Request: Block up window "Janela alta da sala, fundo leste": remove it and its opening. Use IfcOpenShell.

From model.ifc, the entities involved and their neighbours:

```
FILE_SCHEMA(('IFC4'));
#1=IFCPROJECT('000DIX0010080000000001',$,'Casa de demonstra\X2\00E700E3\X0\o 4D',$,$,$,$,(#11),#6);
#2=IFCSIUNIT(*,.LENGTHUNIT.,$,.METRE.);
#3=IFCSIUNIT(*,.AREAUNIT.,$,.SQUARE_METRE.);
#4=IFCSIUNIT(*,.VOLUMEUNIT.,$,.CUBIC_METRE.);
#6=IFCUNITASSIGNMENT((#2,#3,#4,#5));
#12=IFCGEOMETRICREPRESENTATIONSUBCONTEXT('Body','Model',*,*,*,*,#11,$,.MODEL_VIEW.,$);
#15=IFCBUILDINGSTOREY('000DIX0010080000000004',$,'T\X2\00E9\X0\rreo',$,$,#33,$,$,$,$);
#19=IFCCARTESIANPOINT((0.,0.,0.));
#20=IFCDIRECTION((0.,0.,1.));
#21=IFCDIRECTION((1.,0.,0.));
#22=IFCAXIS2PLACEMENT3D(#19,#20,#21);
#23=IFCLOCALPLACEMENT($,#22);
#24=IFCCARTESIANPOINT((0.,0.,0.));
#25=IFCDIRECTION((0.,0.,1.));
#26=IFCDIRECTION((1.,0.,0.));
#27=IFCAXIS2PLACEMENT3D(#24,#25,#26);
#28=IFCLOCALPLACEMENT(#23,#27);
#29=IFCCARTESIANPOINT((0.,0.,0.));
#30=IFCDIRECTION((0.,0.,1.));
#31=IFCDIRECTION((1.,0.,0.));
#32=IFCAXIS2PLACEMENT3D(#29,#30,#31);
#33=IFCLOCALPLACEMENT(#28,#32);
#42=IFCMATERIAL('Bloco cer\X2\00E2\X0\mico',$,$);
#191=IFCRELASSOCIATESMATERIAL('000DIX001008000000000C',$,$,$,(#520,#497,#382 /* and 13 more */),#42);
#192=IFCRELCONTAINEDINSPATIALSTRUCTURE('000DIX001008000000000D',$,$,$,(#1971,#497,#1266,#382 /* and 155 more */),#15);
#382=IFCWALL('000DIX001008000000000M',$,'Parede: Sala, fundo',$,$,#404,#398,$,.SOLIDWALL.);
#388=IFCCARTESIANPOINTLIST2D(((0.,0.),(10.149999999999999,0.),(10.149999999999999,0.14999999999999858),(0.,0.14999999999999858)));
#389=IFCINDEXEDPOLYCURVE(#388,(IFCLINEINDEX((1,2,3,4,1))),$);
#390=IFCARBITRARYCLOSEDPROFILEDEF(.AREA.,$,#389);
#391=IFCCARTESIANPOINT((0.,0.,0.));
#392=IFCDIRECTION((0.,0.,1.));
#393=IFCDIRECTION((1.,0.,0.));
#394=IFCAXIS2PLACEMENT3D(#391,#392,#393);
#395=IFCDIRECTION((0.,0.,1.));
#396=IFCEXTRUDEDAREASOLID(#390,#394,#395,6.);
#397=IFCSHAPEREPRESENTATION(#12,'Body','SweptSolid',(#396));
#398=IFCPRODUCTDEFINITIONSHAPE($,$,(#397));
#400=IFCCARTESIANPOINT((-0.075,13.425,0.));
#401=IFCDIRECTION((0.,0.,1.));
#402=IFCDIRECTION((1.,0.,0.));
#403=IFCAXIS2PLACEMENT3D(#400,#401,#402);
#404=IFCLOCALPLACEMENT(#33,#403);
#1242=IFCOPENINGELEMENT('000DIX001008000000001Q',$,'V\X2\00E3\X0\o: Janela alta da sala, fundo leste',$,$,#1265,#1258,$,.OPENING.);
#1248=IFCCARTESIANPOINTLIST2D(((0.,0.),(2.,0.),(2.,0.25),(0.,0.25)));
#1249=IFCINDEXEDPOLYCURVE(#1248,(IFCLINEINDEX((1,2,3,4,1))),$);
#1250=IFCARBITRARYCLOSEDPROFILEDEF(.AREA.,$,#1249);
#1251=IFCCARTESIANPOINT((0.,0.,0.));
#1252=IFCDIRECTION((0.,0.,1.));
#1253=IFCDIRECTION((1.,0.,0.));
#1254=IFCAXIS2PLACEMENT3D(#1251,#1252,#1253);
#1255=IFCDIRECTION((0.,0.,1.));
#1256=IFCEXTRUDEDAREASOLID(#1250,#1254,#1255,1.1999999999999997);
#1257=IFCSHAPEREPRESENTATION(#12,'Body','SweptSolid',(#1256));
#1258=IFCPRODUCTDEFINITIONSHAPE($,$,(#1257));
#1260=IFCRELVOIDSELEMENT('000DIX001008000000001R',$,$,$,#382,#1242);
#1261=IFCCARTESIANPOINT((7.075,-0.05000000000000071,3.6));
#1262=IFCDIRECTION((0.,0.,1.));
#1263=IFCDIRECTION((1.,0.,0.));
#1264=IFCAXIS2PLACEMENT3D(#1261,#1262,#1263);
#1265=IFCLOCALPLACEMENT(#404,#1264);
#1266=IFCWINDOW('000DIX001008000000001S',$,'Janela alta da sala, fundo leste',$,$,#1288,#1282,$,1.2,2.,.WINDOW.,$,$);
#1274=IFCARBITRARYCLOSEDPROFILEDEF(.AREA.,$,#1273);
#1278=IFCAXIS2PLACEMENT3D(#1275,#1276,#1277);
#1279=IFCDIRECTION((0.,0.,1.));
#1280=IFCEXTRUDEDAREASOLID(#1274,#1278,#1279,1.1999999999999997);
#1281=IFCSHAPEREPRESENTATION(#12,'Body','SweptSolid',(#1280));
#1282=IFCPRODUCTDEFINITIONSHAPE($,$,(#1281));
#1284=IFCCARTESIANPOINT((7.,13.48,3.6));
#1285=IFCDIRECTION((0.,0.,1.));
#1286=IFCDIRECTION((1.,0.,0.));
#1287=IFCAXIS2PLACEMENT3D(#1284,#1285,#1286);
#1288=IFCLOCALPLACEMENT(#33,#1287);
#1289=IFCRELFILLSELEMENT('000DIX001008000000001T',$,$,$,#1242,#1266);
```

```python
import ifcopenshell
import ifcopenshell.api.feature
import ifcopenshell.api.root
import ifcopenshell.geom
import ifcopenshell.util.shape

model = ifcopenshell.open("model.ifc")
settings = ifcopenshell.geom.settings()


def volume(element):
    """Net volume in cubic metres, openings subtracted."""
    shape = ifcopenshell.geom.create_shape(settings, element)
    return ifcopenshell.util.shape.get_volume(shape.geometry)


window = model.by_guid("000DIX001008000000001S")
opening = window.FillsVoids[0].RelatingOpeningElement
wall = opening.VoidsElements[0].RelatingBuildingElement
before = volume(wall)

ifcopenshell.api.root.remove_product(model, product=window)
ifcopenshell.api.feature.remove_feature(model, feature=opening)

after = volume(wall)

print(f"wall volume {before:.3f} -> {after:.3f} m3")

model.write("model-out.ifc")
```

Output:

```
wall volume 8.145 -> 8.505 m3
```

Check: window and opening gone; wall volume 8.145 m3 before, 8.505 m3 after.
